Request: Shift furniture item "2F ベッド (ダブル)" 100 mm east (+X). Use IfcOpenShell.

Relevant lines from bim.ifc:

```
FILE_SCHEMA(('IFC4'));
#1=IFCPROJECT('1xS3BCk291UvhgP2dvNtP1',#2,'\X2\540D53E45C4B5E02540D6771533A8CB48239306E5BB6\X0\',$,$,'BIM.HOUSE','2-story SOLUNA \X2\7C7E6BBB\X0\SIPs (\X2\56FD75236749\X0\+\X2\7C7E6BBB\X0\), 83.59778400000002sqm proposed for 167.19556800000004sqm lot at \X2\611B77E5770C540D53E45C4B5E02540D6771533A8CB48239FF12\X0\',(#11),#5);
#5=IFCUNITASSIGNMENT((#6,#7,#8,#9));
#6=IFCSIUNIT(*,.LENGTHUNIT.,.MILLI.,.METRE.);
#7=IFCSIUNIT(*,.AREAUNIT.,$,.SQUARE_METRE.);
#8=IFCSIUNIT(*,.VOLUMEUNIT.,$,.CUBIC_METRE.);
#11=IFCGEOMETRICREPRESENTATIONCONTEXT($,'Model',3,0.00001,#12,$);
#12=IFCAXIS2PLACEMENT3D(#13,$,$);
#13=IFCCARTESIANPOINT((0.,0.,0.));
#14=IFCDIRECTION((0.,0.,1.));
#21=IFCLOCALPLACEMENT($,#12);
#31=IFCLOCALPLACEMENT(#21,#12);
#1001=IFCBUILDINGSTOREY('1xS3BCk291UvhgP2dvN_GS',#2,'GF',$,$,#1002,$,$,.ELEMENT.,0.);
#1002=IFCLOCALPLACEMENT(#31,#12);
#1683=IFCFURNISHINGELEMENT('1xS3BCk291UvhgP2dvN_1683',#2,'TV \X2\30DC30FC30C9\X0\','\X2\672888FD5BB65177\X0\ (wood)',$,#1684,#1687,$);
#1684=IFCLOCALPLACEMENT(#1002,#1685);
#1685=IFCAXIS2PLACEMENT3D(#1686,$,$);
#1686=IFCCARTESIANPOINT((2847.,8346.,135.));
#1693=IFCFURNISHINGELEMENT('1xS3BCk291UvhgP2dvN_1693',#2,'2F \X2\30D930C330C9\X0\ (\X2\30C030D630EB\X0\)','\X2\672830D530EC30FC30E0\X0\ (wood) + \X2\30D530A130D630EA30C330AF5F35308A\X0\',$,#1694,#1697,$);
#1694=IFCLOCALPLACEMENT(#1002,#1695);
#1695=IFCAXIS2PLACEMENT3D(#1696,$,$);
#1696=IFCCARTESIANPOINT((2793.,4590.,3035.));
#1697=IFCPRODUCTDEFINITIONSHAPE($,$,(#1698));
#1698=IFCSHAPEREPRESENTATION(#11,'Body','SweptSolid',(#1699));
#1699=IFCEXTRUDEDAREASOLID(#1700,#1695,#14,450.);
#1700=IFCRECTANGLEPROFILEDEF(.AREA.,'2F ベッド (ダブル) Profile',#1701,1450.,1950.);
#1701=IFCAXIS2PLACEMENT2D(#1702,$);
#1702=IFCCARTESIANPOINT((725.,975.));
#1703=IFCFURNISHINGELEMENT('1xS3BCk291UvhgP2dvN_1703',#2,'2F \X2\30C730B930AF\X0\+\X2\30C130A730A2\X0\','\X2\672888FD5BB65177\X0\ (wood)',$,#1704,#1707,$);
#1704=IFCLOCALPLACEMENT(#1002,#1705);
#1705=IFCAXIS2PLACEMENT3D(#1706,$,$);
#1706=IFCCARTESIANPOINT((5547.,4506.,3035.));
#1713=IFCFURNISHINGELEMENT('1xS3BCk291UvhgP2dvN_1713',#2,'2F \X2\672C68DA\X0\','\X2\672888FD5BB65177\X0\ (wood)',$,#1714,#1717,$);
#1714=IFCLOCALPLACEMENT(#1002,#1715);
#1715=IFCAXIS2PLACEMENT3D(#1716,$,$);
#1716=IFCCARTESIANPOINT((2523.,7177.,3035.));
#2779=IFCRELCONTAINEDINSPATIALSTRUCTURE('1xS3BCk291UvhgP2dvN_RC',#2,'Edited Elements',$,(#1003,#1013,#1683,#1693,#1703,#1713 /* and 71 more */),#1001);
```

```python
import ifcopenshell
import ifcopenshell.api.geometry
import ifcopenshell.util.placement
import ifcopenshell.util.unit

model = ifcopenshell.open("bim.ifc")
unit_scale = ifcopenshell.util.unit.calculate_unit_scale(model)

item = model.by_guid("1xS3BCk291UvhgP2dvN_1693")
matrix = ifcopenshell.util.placement.get_local_placement(item.ObjectPlacement)
matrix[0, 3] += 0.1 / unit_scale
ifcopenshell.api.geometry.edit_object_placement(model, product=item, matrix=matrix, is_si=False)

print(ifcopenshell.util.placement.get_local_placement(item.ObjectPlacement).round(3) + 0.0)

model.write("bim_rev.ifc")
```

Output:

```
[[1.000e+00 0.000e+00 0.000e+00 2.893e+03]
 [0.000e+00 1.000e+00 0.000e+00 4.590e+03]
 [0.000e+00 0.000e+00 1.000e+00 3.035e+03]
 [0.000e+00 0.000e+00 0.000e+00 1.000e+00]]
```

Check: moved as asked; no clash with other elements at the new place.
